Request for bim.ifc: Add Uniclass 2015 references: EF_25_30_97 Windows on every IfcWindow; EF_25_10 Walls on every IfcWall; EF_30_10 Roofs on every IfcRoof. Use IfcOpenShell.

First a look at what the model holds.

```python
import ifcopenshell

model = ifcopenshell.open("bim.ifc")
print(model.schema)
print("classifications:", [c.Name for c in model.by_type("IfcClassification")])
for ifc_class in ("IfcDoor", "IfcRoof", "IfcStair", "IfcWall", "IfcWindow"):
    print(ifc_class, len(model.by_type(ifc_class)))
```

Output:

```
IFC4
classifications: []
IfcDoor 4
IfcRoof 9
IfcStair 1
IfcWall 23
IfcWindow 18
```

```python
import ifcopenshell
import ifcopenshell.api.classification

model = ifcopenshell.open("bim.ifc")

system = ifcopenshell.api.classification.add_classification(model, classification="Uniclass 2015")

codes = {
    "IfcWindow": ("EF_25_30_97", "Windows"),
    "IfcWall": ("EF_25_10", "Walls"),
    "IfcRoof": ("EF_30_10", "Roofs"),
}
for ifc_class, (code, name) in codes.items():
    products = model.by_type(ifc_class)
    ifcopenshell.api.classification.add_reference(
        model, products=products, classification=system, identification=code, name=name
    )
    print(code, len(products))

model.write("bim_rev.ifc")
```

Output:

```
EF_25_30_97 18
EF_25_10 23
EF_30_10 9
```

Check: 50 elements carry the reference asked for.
